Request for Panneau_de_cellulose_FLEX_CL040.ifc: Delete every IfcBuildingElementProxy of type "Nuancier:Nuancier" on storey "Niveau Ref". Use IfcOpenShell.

First a look at what the model holds.

```python
import ifcopenshell
import ifcopenshell.util.element

model = ifcopenshell.open("Panneau_de_cellulose_FLEX_CL040.ifc")
print(model.schema)
storey = next(s for s in model.by_type("IfcBuildingStorey") if s.Name == "Niveau Ref")
proxies = [e for e in ifcopenshell.util.element.get_decomposition(storey) if e.is_a("IfcBuildingElementProxy")]
seen = {}
for e in proxies:
    element_type = ifcopenshell.util.element.get_type(e)
    name = element_type.Name if element_type not in (None, e) else None
    seen[name] = seen.get(name, 0) + 1
for name, count in sorted(seen.items(), key=str):
    print(count, "x", name)
```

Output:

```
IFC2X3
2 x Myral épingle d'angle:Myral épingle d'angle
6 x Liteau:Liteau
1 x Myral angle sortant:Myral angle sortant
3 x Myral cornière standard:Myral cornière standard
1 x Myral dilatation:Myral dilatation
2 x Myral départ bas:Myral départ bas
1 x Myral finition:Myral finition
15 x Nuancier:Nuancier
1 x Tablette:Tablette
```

```python
import ifcopenshell
import ifcopenshell.api.root
import ifcopenshell.util.element

model = ifcopenshell.open("Panneau_de_cellulose_FLEX_CL040.ifc")

storey = next(s for s in model.by_type("IfcBuildingStorey") if s.Name == "Niveau Ref")
proxies = [e for e in ifcopenshell.util.element.get_decomposition(storey) if e.is_a("IfcBuildingElementProxy")]
targets = [e for e in proxies if (t := ifcopenshell.util.element.get_type(e)) not in (None, e) and t.Name == "Nuancier:Nuancier"]

for e in targets:
    ifcopenshell.api.root.remove_product(model, product=e)
print(len(targets), "removed")

model.write("Panneau_de_cellulose_FLEX_CL040-out.ifc")
```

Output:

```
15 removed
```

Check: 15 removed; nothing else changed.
